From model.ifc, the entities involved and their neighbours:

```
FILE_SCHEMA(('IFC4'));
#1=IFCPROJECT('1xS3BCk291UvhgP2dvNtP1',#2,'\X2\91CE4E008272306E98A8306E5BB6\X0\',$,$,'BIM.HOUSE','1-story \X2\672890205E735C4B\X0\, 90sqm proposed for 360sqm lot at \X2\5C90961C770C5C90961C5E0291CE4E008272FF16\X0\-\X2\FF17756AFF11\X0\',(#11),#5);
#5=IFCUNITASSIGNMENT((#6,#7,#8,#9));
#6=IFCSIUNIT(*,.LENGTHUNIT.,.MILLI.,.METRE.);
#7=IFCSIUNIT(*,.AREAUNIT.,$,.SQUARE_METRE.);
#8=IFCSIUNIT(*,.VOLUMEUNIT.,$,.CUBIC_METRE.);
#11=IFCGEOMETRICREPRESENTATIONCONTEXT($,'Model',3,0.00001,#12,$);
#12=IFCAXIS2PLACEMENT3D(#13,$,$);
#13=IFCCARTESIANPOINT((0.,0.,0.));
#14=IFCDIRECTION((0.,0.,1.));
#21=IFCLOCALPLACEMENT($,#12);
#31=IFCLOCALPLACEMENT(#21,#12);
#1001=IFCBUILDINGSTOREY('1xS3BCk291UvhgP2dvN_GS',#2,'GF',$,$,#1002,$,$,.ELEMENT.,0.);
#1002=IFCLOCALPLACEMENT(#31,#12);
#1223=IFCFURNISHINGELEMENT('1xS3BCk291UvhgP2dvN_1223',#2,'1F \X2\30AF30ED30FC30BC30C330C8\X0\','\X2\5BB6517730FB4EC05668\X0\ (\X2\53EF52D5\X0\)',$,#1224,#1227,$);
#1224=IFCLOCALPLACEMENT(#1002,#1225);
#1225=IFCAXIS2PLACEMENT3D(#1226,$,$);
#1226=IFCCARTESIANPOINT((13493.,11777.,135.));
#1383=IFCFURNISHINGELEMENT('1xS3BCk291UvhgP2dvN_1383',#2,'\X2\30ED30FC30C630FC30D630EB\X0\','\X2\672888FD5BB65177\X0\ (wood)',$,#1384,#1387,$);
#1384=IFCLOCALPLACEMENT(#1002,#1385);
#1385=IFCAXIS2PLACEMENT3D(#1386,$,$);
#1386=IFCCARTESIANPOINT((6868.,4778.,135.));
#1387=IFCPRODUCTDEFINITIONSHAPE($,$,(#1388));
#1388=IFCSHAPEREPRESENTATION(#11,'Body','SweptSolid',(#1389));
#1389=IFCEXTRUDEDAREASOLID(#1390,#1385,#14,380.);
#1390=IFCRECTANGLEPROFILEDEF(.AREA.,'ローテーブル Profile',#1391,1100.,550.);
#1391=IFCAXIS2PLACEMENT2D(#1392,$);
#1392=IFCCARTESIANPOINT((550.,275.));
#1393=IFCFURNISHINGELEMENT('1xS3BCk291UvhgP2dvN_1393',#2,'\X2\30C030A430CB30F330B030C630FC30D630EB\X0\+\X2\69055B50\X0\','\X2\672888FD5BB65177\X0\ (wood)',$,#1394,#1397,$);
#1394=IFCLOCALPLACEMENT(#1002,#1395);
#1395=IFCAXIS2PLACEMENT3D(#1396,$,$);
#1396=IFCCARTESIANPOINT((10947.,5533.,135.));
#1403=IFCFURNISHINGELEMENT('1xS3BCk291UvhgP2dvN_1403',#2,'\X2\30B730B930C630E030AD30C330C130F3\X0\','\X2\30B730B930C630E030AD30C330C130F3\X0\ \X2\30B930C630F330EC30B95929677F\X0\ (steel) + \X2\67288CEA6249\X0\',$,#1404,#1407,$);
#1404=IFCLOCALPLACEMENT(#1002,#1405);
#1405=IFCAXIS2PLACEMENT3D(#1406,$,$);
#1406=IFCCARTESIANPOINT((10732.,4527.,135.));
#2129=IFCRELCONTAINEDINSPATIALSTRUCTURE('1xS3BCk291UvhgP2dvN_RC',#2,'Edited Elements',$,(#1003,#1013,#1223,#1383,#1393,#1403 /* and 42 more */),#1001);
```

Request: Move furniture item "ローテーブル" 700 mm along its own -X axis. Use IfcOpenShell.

```python
import ifcopenshell
import ifcopenshell.api.geometry
import ifcopenshell.util.placement

model = ifcopenshell.open("model.ifc")

item = model.by_guid("1xS3BCk291UvhgP2dvN_1383")
matrix = ifcopenshell.util.placement.get_local_placement(item.ObjectPlacement)
matrix[:3, 3] -= matrix[:3, 0] * 700.0
ifcopenshell.api.geometry.edit_object_placement(model, product=item, matrix=matrix, is_si=False)

print(ifcopenshell.util.placement.get_local_placement(item.ObjectPlacement).round(3) + 0.0)

model.write("model-out.ifc")
```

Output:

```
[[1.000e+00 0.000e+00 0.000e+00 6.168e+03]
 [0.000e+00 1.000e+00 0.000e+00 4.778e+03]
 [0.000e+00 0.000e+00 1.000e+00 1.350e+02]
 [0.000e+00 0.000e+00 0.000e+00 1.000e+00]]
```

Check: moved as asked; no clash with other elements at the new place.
